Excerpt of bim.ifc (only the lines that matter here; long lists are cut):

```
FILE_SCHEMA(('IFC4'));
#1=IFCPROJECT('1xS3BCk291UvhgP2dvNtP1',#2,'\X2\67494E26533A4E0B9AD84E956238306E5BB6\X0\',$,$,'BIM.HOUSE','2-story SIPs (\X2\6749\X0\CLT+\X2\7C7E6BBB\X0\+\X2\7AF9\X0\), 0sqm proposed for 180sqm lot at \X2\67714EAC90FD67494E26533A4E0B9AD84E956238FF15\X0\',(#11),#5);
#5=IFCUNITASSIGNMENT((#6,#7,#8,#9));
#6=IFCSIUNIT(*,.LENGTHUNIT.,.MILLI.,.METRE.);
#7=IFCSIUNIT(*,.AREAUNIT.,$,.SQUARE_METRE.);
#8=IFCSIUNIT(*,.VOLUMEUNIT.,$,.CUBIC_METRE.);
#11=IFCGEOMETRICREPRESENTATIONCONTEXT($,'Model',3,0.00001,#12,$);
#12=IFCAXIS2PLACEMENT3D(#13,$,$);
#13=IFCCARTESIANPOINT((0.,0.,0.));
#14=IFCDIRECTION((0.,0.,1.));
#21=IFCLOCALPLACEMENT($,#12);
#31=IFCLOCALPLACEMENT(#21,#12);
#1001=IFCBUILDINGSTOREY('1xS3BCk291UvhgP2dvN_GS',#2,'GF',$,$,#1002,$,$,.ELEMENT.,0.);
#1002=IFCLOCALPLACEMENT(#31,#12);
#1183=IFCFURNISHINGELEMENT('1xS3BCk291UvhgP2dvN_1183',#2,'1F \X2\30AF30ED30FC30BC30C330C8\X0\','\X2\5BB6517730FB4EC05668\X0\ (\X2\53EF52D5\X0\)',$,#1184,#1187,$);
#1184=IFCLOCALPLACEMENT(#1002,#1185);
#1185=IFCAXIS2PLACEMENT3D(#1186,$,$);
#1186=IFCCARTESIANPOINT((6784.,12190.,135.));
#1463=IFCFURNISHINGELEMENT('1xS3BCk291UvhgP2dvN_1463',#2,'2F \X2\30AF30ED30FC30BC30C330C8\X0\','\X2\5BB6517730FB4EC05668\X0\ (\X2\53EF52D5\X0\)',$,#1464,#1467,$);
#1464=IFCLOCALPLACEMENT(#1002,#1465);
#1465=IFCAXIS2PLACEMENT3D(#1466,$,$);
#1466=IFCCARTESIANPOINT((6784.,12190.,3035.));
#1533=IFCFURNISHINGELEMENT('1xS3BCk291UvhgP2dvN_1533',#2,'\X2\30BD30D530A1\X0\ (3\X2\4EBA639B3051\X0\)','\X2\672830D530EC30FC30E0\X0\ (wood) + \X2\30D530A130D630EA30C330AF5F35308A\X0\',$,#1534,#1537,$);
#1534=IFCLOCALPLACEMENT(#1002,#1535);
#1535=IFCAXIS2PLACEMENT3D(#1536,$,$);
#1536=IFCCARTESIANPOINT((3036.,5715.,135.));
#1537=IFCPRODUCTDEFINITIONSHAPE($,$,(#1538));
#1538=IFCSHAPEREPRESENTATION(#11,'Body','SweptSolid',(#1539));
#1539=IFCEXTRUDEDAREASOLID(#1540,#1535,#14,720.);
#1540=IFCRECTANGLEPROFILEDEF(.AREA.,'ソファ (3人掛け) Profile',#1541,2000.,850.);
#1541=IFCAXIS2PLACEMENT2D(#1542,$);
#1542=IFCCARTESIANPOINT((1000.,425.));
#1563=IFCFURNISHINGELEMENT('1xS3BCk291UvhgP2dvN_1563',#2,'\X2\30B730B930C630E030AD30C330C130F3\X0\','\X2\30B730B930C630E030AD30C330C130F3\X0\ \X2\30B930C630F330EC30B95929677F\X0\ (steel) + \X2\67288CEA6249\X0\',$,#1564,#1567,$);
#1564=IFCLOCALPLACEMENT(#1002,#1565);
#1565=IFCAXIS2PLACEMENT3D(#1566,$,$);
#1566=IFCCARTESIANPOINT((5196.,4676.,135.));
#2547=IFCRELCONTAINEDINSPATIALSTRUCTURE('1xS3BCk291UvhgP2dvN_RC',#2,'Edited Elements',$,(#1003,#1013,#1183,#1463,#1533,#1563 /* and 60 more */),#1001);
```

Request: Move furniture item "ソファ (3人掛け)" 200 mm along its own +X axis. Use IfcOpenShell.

```python
import ifcopenshell
import ifcopenshell.api.geometry
import ifcopenshell.util.placement
import ifcopenshell.util.unit

model = ifcopenshell.open("bim.ifc")
unit_scale = ifcopenshell.util.unit.calculate_unit_scale(model)

item = model.by_guid("1xS3BCk291UvhgP2dvN_1533")
matrix = ifcopenshell.util.placement.get_local_placement(item.ObjectPlacement)
matrix[:3, 3] += matrix[:3, 0] * 0.2 / unit_scale
ifcopenshell.api.geometry.edit_object_placement(model, product=item, matrix=matrix, is_si=False)

print(ifcopenshell.util.placement.get_local_placement(item.ObjectPlacement).round(3) + 0.0)

model.write("bim_updated.ifc")
```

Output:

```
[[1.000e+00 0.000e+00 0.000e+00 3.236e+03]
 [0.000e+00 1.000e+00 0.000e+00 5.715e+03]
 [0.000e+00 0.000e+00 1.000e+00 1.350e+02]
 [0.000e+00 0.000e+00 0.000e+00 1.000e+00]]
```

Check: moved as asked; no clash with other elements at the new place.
